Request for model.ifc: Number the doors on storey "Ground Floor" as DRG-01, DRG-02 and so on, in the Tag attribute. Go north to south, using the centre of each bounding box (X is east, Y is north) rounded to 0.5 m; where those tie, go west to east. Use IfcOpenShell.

First a look at what the model holds.

```python
import ifcopenshell
import ifcopenshell.util.element
import ifcopenshell.util.placement

model = ifcopenshell.open("model.ifc")
print(model.schema)
storey = next(s for s in model.by_type("IfcBuildingStorey") if s.Name == "Ground Floor")
doors = [e for e in ifcopenshell.util.element.get_decomposition(storey) if e.is_a("IfcDoor")]
for e in sorted(doors, key=lambda e: e.id()):
    origin = ifcopenshell.util.placement.get_local_placement(e.ObjectPlacement)[:3, 3]
    print(e.id(), e.Tag, e.Name, origin.round(2) + 0.0, sep=" | ")
```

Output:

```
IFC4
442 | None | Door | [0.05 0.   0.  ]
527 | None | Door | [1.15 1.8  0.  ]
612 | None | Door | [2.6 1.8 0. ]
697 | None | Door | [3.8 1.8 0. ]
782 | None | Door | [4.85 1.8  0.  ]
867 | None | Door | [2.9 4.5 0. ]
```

```python
import ifcopenshell
import ifcopenshell.geom
import ifcopenshell.util.element
import ifcopenshell.util.shape

model = ifcopenshell.open("model.ifc")
settings = ifcopenshell.geom.settings()
settings.set("use-world-coords", True)


def centre(element):
    shape = ifcopenshell.geom.create_shape(settings, element)
    return ifcopenshell.util.shape.get_bbox_centroid(shape.geometry)


storey = next(s for s in model.by_type("IfcBuildingStorey") if s.Name == "Ground Floor")
doors = [e for e in ifcopenshell.util.element.get_decomposition(storey) if e.is_a("IfcDoor")]

# Insertion points can sit at a corner or the storey origin, so sort by the geometry (in metres).
centres = {e: centre(e) for e in doors}
doors.sort(key=lambda e: (-round(centres[e][1] / 0.5), centres[e][0]))

for i, e in enumerate(doors, start=1):
    number = f"DRG-{i:02d}"
    e.Tag = number
    print(e.id(), number)

model.write("model_updated.ifc")
```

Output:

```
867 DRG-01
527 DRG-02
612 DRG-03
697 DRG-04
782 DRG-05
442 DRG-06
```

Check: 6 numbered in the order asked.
